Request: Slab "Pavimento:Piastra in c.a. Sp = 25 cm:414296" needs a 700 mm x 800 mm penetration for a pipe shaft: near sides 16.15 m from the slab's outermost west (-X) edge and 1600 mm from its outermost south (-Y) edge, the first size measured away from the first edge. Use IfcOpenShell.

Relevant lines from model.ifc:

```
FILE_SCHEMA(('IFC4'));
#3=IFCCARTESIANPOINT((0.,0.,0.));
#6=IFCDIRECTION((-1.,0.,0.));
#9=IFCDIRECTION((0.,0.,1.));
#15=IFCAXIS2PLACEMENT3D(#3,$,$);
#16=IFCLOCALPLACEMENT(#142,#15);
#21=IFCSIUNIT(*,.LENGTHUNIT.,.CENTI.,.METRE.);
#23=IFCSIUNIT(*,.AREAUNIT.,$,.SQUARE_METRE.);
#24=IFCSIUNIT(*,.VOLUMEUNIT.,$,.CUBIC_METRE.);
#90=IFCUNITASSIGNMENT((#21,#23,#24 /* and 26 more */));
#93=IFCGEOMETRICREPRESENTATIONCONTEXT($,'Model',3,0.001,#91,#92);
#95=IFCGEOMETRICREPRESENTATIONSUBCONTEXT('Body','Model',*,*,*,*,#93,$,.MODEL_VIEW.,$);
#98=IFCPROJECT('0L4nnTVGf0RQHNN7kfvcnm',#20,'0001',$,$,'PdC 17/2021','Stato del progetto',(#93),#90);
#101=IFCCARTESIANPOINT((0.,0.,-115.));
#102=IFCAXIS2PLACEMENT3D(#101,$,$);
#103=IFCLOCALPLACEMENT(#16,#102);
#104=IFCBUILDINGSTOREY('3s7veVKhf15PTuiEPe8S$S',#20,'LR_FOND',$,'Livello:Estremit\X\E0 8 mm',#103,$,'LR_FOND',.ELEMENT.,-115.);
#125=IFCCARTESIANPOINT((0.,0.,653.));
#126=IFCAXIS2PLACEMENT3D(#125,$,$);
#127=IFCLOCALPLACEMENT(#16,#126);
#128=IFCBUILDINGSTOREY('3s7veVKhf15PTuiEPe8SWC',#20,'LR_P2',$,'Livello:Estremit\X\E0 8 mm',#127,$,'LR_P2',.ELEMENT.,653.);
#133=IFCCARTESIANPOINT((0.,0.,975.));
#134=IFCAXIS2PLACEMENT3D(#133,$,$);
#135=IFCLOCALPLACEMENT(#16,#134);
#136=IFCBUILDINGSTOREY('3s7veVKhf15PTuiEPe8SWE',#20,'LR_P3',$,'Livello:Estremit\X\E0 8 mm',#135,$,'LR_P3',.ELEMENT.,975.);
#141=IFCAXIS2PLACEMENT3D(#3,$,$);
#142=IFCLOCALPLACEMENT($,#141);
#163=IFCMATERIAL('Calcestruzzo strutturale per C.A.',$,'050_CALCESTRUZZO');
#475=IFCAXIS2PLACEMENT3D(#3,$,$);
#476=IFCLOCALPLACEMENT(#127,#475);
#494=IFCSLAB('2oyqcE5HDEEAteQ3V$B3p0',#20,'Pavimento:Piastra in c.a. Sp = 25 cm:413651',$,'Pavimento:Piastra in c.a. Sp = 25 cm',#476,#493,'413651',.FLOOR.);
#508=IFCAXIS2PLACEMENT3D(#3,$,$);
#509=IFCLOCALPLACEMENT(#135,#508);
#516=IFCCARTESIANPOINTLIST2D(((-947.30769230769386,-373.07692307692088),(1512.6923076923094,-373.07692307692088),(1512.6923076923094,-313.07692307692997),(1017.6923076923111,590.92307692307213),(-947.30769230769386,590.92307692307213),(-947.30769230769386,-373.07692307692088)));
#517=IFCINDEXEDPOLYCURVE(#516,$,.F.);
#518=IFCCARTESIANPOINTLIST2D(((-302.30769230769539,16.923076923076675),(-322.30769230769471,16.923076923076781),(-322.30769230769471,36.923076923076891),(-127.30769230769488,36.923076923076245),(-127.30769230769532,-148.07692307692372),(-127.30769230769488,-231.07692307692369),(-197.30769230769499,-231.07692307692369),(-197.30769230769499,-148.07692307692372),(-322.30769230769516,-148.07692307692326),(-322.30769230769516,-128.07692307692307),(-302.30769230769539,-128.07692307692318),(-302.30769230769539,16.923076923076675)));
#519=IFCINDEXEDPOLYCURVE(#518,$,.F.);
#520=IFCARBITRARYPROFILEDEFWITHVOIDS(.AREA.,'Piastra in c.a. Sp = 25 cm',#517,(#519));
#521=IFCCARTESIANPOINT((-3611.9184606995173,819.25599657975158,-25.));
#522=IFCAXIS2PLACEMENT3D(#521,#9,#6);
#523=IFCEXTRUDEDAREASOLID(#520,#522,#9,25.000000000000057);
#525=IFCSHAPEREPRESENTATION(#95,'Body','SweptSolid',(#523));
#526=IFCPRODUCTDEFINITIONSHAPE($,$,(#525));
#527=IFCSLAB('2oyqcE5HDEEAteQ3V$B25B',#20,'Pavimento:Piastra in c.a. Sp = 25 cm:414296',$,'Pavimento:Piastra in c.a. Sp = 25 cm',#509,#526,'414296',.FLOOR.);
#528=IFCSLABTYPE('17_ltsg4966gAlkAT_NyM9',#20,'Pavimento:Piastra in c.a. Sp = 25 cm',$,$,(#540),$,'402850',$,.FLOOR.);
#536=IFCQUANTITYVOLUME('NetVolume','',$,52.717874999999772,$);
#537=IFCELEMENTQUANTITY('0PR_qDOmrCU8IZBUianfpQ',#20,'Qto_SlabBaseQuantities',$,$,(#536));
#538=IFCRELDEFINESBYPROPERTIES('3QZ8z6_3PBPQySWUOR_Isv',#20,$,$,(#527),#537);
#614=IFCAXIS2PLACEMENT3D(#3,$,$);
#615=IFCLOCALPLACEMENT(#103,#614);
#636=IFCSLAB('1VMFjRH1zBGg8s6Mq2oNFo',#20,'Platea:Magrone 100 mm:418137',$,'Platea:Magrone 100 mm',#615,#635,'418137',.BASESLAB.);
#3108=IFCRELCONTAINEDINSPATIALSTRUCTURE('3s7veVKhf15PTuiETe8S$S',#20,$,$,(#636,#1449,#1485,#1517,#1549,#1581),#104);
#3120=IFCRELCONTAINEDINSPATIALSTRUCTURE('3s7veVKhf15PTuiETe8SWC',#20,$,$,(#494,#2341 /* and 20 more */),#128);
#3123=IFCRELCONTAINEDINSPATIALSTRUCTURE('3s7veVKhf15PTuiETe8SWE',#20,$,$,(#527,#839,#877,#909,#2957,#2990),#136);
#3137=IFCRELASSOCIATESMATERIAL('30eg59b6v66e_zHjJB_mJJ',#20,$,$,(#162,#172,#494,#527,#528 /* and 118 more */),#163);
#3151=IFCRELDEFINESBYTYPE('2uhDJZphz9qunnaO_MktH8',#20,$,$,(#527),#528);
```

```python
import numpy as np
import ifcopenshell
import ifcopenshell.api.feature
import ifcopenshell.api.geometry
import ifcopenshell.api.pset
import ifcopenshell.api.root
import ifcopenshell.geom
import ifcopenshell.util.element
import ifcopenshell.util.placement
import ifcopenshell.util.representation
import ifcopenshell.util.shape
import ifcopenshell.util.unit

model = ifcopenshell.open("model.ifc")
unit_scale = ifcopenshell.util.unit.calculate_unit_scale(model)
volume_scale = ifcopenshell.util.unit.calculate_unit_scale(model, "VOLUMEUNIT")
settings = ifcopenshell.geom.settings()


def volume(element):
    """Net volume in cubic metres, openings subtracted."""
    shape = ifcopenshell.geom.create_shape(settings, element)
    return ifcopenshell.util.shape.get_volume(shape.geometry)


slab = model.by_guid("2oyqcE5HDEEAteQ3V$B25B")
before = volume(slab)

# Extent in the slab's own axes, in metres. The edges named are its -X and -Y sides.
slab_shape = ifcopenshell.geom.create_shape(settings, slab)
vertices = ifcopenshell.util.shape.get_vertices(slab_shape.geometry)
x_min, y_min, bottom = vertices.min(axis=0)
top = vertices[:, 2].max()

opening = ifcopenshell.api.root.create_entity(model, ifc_class="IfcOpeningElement", name="Pipe shaft opening", predefined_type="OPENING")
context = ifcopenshell.util.representation.get_context(model, "Model", "Body", "MODEL_VIEW")
width, depth = 0.7, 0.8
outline = [(0.0, 0.0), (width, 0.0), (width, depth), (0.0, depth), (0.0, 0.0)]
# Overshoot both faces by 50 mm so the cut is clean.
shape = ifcopenshell.api.geometry.add_slab_representation(
    model, context=context, depth=top - bottom + 0.1, polyline=outline
)
ifcopenshell.api.geometry.assign_representation(model, product=opening, representation=shape)

matrix = ifcopenshell.util.placement.get_local_placement(slab.ObjectPlacement)
matrix[:, 3] = matrix @ np.append(np.array([x_min + 16.15, y_min + 1.6, bottom - 0.05]) / unit_scale, 1.0)
ifcopenshell.api.geometry.edit_object_placement(model, product=opening, matrix=matrix, is_si=False)
ifcopenshell.api.feature.add_feature(model, feature=opening, element=slab)

after = volume(slab)

# Update the slab's stored quantities.
qto = model.by_id(ifcopenshell.util.element.get_pset(slab, "Qto_SlabBaseQuantities", should_inherit=False)["id"])
ifcopenshell.api.pset.edit_qto(model, qto=qto, properties={"NetVolume": after / volume_scale})

print(f"slab volume {before:.3f} -> {after:.3f} m3")

model.write("model_rev.ifc")
```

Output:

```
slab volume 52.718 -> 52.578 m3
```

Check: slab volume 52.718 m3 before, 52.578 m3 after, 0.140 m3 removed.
